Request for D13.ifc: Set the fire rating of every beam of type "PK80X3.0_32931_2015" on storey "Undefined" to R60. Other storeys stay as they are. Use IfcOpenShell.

First a look at what the model holds.

```python
import ifcopenshell
import ifcopenshell.util.element

model = ifcopenshell.open("D13.ifc")
print(model.schema)
storey = next(s for s in model.by_type("IfcBuildingStorey") if s.Name == "Undefined")
beams = [e for e in ifcopenshell.util.element.get_decomposition(storey) if e.is_a("IfcBeam")]
seen = {}
for e in beams:
    element_type = ifcopenshell.util.element.get_type(e)
    key = (element_type.Name if element_type != e and element_type else None, ifcopenshell.util.element.get_pset(e, "Pset_BeamCommon", "FireRating"))
    seen[key] = seen.get(key, 0) + 1
for (name, value), count in sorted(seen.items(), key=str):
    print(count, "x", name, "|", value)
```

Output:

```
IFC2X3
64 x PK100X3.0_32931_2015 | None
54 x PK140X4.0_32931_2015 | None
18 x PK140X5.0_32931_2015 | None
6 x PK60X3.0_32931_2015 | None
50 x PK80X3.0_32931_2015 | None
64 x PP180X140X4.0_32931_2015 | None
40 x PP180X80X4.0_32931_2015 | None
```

```python
import ifcopenshell
import ifcopenshell.api.pset
import ifcopenshell.util.element

model = ifcopenshell.open("D13.ifc")

storey = next(s for s in model.by_type("IfcBuildingStorey") if s.Name == "Undefined")
beams = [e for e in ifcopenshell.util.element.get_decomposition(storey) if e.is_a("IfcBeam")]

count = 0
for e in beams:
    element_type = ifcopenshell.util.element.get_type(e)
    if element_type in (None, e) or element_type.Name != "PK80X3.0_32931_2015":
        continue
    found = ifcopenshell.util.element.get_pset(e, "Pset_BeamCommon", should_inherit=False)
    if found:
        pset = model.by_id(found["id"])
        if len(ifcopenshell.util.element.get_elements_by_pset(pset)) > 1:
            pset = ifcopenshell.api.pset.unshare_pset(model, products=[e], pset=pset)[0]
    else:
        pset = ifcopenshell.api.pset.add_pset(model, product=e, name="Pset_BeamCommon")
    ifcopenshell.api.pset.edit_pset(model, pset=pset, properties={"FireRating": "R60"})
    count += 1

print(count, "beams updated")

model.write("D13_v2.ifc")
```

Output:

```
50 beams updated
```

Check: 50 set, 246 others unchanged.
